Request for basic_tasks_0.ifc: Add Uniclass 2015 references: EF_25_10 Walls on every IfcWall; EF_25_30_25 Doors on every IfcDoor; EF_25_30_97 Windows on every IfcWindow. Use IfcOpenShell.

First a look at what the model holds.

```python
import ifcopenshell

model = ifcopenshell.open("basic_tasks_0.ifc")
print(model.schema)
print("classifications:", [c.Name for c in model.by_type("IfcClassification")])
for ifc_class in ("IfcDoor", "IfcRoof", "IfcStair", "IfcWall", "IfcWindow"):
    print(ifc_class, len(model.by_type(ifc_class)))
```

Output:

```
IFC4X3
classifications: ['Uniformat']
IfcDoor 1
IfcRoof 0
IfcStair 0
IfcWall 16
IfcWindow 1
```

```python
import ifcopenshell
import ifcopenshell.api.classification

model = ifcopenshell.open("basic_tasks_0.ifc")

system = ifcopenshell.api.classification.add_classification(model, classification="Uniclass 2015")

codes = {
    "IfcWall": ("EF_25_10", "Walls"),
    "IfcDoor": ("EF_25_30_25", "Doors"),
    "IfcWindow": ("EF_25_30_97", "Windows"),
}
for ifc_class, (code, name) in codes.items():
    products = model.by_type(ifc_class)
    ifcopenshell.api.classification.add_reference(
        model, products=products, classification=system, identification=code, name=name
    )
    print(code, len(products))

model.write("basic_tasks_0_edited.ifc")
```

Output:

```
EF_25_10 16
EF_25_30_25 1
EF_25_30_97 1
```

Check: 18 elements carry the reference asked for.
